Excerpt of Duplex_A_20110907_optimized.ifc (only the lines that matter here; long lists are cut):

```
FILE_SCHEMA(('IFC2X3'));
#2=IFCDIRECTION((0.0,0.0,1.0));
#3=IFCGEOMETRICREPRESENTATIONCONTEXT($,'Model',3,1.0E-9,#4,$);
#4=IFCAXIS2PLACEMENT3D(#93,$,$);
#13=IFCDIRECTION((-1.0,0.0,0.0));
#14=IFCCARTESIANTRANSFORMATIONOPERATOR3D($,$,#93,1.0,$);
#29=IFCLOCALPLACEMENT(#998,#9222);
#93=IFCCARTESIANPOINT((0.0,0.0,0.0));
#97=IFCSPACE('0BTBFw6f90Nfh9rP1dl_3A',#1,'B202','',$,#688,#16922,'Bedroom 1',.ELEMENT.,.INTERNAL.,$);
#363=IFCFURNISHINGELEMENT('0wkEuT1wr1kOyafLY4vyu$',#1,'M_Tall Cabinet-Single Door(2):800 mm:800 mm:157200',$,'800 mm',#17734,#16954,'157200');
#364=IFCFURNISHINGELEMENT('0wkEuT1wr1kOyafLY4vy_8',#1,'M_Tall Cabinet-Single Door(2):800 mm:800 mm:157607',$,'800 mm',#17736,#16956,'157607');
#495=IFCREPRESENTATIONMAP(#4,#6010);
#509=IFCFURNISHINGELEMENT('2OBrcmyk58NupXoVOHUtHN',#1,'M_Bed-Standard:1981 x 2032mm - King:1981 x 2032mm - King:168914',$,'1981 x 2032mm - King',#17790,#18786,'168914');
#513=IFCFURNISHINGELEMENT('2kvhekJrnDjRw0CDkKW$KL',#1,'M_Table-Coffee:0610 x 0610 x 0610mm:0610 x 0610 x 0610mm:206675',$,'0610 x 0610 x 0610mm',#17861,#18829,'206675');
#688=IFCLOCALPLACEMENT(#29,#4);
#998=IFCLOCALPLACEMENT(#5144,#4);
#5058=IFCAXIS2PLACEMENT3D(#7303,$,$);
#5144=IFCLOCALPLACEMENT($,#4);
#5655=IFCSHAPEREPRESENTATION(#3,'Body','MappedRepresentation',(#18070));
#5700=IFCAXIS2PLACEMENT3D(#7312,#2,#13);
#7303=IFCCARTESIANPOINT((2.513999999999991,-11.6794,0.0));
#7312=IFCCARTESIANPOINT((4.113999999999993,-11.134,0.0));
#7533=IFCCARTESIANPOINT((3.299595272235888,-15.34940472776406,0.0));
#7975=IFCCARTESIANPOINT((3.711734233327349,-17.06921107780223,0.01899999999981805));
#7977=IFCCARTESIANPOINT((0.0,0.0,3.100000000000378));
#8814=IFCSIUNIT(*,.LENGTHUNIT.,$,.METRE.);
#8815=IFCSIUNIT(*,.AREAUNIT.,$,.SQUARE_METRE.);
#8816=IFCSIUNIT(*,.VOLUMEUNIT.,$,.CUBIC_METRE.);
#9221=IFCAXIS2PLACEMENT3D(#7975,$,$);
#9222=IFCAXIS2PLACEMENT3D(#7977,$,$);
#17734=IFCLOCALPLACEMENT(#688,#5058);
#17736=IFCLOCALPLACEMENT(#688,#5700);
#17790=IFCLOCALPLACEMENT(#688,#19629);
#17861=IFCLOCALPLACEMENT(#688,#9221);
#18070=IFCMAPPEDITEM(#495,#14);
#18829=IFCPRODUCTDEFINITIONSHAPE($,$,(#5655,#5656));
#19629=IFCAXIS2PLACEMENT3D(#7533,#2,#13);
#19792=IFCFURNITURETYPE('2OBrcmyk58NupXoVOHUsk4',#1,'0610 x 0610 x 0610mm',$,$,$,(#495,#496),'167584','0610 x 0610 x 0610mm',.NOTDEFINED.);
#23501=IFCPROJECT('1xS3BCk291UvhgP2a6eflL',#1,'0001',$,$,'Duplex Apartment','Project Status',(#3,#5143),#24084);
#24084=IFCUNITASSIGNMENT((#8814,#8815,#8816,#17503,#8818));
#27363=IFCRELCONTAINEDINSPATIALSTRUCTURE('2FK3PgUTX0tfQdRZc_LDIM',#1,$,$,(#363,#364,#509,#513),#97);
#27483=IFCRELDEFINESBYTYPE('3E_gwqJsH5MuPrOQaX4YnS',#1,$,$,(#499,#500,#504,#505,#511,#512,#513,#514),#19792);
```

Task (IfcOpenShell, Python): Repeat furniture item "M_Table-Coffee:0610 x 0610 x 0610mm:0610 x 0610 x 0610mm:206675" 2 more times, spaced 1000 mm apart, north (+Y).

```python
import numpy as np
import ifcopenshell
import ifcopenshell.api.geometry
import ifcopenshell.api.root
import ifcopenshell.util.element
import ifcopenshell.util.placement

model = ifcopenshell.open("Duplex_A_20110907_optimized.ifc")


def reuse_history(source, copy):
    """copy_class also copies each property set's owner history, people and application; keep the originals."""
    for rel in copy.IsDefinedBy:
        if rel.is_a("IfcRelDefinesByProperties") and (history := rel.RelatingPropertyDefinition.OwnerHistory):
            rel.RelatingPropertyDefinition.OwnerHistory = source.OwnerHistory
            ifcopenshell.util.element.remove_deep2(model, history)


source = model.by_id(513)
base = ifcopenshell.util.placement.get_local_placement(source.ObjectPlacement)
step = np.array([0.0, 1.0, 0.0]) * 1.0

for i in range(1, 3):
    copy = ifcopenshell.api.root.copy_class(model, product=source)
    copy.Representation = ifcopenshell.util.element.copy_deep(
        model, source.Representation, exclude=["IfcGeometricRepresentationContext", "IfcRepresentationMap"]
    )
    copy.Name = "M_Table-Coffee:0610 x 0610 x 0610mm:0610 x 0610 x 0610mm"
    copy.Tag = None
    reuse_history(source, copy)
    matrix = base.copy()
    matrix[:3, 3] += i * step
    print("added at", matrix[:3, 3].round(3) + 0.0)
    ifcopenshell.api.geometry.edit_object_placement(model, product=copy, matrix=matrix, is_si=False)

model.write("Duplex_A_20110907_optimized-out.ifc")
```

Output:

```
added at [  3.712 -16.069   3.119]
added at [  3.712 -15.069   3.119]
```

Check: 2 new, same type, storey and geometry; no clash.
